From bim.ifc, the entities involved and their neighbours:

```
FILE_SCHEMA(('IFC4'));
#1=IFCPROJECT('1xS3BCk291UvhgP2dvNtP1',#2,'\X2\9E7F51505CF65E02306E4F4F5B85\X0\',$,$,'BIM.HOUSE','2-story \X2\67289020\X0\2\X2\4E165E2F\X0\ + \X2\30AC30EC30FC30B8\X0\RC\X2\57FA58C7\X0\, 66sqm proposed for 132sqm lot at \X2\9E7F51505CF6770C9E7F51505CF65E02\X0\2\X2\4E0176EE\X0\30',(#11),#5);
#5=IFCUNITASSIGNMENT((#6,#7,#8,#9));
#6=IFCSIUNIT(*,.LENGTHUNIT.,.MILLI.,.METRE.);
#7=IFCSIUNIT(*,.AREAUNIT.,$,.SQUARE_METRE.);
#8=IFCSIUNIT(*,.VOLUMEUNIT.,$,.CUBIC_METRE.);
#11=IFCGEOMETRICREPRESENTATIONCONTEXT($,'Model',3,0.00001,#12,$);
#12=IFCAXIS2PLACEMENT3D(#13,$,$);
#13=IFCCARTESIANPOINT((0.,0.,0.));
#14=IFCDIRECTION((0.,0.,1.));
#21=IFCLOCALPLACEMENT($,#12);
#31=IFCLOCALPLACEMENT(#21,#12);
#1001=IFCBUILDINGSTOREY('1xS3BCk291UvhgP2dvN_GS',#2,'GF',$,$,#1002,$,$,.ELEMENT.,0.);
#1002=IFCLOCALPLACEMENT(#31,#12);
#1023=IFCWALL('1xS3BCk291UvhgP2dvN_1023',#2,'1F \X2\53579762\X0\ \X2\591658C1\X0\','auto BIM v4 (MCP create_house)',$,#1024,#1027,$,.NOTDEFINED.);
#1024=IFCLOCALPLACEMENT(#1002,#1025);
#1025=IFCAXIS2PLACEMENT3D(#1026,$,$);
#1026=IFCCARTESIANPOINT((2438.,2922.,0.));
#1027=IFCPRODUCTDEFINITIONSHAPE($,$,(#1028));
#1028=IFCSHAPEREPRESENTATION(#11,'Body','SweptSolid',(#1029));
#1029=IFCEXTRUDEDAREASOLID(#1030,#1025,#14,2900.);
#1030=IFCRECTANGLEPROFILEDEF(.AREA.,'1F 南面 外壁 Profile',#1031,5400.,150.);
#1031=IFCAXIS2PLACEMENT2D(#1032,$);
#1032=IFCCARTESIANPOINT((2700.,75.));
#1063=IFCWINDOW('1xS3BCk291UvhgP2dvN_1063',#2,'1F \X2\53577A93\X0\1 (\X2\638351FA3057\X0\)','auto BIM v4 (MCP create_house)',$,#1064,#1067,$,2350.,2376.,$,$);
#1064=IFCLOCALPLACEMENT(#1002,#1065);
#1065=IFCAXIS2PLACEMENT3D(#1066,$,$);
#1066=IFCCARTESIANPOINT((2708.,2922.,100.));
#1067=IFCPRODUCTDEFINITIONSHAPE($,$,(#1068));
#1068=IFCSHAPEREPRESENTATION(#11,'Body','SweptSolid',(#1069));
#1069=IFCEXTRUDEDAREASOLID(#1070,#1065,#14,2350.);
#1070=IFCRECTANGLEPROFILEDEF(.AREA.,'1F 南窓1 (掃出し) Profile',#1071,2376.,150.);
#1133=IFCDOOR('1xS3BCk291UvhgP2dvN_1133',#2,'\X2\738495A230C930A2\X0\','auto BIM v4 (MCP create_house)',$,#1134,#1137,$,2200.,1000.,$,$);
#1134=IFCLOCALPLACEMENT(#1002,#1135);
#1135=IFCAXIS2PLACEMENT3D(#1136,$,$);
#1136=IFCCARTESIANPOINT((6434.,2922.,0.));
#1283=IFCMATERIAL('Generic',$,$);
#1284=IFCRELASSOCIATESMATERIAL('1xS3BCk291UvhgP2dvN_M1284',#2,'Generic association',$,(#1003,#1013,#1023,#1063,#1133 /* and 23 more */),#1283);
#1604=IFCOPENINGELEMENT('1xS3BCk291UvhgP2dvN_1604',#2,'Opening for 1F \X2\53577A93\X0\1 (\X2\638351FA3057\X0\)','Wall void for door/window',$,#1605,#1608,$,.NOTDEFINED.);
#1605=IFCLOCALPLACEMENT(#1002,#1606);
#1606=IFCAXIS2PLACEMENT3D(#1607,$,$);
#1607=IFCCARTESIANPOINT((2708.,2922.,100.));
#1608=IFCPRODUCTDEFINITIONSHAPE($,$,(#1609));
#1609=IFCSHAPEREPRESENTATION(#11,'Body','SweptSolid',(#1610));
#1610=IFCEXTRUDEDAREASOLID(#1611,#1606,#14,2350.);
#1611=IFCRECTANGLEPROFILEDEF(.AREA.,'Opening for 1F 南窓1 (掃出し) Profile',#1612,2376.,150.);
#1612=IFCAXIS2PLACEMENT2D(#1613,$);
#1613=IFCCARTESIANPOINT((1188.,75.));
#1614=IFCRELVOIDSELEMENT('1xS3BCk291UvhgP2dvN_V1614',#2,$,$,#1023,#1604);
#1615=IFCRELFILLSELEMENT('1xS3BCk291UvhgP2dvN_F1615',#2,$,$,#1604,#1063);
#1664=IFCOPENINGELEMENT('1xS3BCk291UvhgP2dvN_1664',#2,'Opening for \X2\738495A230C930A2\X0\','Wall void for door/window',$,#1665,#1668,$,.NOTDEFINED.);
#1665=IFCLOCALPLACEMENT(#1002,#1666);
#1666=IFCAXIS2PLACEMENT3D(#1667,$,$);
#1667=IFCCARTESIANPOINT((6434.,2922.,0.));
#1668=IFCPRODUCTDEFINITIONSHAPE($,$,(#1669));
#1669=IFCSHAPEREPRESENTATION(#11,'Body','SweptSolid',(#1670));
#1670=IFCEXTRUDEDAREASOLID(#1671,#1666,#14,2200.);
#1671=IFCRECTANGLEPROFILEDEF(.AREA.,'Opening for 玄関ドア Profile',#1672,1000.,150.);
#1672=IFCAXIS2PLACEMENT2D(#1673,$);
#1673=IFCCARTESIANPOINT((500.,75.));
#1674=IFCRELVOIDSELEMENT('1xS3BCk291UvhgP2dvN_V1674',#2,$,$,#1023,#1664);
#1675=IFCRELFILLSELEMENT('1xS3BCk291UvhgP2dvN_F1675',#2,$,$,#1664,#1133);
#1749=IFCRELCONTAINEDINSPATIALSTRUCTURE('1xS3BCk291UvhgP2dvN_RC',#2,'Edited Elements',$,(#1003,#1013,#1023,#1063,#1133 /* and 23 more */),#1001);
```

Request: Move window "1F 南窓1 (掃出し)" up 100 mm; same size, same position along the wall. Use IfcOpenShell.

```python
import numpy as np
import ifcopenshell
import ifcopenshell.api.geometry
import ifcopenshell.util.placement
import ifcopenshell.util.unit

model = ifcopenshell.open("bim.ifc")
unit_scale = ifcopenshell.util.unit.calculate_unit_scale(model)

window = model.by_id(1063)
opening = window.FillsVoids[0].RelatingOpeningElement
dz = 100.0

shift = np.array([0.0, 0.0, dz])
# The window is not placed relative to its opening, so move both.
for product in (opening, window):
    matrix = ifcopenshell.util.placement.get_local_placement(product.ObjectPlacement)
    matrix[:3, 3] += shift
    ifcopenshell.api.geometry.edit_object_placement(model, product=product, matrix=matrix, is_si=False)

print(f"moved by {dz * unit_scale:+.3f} m")

model.write("bim_edited.ifc")
```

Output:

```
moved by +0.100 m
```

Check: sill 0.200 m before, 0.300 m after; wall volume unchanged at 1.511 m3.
